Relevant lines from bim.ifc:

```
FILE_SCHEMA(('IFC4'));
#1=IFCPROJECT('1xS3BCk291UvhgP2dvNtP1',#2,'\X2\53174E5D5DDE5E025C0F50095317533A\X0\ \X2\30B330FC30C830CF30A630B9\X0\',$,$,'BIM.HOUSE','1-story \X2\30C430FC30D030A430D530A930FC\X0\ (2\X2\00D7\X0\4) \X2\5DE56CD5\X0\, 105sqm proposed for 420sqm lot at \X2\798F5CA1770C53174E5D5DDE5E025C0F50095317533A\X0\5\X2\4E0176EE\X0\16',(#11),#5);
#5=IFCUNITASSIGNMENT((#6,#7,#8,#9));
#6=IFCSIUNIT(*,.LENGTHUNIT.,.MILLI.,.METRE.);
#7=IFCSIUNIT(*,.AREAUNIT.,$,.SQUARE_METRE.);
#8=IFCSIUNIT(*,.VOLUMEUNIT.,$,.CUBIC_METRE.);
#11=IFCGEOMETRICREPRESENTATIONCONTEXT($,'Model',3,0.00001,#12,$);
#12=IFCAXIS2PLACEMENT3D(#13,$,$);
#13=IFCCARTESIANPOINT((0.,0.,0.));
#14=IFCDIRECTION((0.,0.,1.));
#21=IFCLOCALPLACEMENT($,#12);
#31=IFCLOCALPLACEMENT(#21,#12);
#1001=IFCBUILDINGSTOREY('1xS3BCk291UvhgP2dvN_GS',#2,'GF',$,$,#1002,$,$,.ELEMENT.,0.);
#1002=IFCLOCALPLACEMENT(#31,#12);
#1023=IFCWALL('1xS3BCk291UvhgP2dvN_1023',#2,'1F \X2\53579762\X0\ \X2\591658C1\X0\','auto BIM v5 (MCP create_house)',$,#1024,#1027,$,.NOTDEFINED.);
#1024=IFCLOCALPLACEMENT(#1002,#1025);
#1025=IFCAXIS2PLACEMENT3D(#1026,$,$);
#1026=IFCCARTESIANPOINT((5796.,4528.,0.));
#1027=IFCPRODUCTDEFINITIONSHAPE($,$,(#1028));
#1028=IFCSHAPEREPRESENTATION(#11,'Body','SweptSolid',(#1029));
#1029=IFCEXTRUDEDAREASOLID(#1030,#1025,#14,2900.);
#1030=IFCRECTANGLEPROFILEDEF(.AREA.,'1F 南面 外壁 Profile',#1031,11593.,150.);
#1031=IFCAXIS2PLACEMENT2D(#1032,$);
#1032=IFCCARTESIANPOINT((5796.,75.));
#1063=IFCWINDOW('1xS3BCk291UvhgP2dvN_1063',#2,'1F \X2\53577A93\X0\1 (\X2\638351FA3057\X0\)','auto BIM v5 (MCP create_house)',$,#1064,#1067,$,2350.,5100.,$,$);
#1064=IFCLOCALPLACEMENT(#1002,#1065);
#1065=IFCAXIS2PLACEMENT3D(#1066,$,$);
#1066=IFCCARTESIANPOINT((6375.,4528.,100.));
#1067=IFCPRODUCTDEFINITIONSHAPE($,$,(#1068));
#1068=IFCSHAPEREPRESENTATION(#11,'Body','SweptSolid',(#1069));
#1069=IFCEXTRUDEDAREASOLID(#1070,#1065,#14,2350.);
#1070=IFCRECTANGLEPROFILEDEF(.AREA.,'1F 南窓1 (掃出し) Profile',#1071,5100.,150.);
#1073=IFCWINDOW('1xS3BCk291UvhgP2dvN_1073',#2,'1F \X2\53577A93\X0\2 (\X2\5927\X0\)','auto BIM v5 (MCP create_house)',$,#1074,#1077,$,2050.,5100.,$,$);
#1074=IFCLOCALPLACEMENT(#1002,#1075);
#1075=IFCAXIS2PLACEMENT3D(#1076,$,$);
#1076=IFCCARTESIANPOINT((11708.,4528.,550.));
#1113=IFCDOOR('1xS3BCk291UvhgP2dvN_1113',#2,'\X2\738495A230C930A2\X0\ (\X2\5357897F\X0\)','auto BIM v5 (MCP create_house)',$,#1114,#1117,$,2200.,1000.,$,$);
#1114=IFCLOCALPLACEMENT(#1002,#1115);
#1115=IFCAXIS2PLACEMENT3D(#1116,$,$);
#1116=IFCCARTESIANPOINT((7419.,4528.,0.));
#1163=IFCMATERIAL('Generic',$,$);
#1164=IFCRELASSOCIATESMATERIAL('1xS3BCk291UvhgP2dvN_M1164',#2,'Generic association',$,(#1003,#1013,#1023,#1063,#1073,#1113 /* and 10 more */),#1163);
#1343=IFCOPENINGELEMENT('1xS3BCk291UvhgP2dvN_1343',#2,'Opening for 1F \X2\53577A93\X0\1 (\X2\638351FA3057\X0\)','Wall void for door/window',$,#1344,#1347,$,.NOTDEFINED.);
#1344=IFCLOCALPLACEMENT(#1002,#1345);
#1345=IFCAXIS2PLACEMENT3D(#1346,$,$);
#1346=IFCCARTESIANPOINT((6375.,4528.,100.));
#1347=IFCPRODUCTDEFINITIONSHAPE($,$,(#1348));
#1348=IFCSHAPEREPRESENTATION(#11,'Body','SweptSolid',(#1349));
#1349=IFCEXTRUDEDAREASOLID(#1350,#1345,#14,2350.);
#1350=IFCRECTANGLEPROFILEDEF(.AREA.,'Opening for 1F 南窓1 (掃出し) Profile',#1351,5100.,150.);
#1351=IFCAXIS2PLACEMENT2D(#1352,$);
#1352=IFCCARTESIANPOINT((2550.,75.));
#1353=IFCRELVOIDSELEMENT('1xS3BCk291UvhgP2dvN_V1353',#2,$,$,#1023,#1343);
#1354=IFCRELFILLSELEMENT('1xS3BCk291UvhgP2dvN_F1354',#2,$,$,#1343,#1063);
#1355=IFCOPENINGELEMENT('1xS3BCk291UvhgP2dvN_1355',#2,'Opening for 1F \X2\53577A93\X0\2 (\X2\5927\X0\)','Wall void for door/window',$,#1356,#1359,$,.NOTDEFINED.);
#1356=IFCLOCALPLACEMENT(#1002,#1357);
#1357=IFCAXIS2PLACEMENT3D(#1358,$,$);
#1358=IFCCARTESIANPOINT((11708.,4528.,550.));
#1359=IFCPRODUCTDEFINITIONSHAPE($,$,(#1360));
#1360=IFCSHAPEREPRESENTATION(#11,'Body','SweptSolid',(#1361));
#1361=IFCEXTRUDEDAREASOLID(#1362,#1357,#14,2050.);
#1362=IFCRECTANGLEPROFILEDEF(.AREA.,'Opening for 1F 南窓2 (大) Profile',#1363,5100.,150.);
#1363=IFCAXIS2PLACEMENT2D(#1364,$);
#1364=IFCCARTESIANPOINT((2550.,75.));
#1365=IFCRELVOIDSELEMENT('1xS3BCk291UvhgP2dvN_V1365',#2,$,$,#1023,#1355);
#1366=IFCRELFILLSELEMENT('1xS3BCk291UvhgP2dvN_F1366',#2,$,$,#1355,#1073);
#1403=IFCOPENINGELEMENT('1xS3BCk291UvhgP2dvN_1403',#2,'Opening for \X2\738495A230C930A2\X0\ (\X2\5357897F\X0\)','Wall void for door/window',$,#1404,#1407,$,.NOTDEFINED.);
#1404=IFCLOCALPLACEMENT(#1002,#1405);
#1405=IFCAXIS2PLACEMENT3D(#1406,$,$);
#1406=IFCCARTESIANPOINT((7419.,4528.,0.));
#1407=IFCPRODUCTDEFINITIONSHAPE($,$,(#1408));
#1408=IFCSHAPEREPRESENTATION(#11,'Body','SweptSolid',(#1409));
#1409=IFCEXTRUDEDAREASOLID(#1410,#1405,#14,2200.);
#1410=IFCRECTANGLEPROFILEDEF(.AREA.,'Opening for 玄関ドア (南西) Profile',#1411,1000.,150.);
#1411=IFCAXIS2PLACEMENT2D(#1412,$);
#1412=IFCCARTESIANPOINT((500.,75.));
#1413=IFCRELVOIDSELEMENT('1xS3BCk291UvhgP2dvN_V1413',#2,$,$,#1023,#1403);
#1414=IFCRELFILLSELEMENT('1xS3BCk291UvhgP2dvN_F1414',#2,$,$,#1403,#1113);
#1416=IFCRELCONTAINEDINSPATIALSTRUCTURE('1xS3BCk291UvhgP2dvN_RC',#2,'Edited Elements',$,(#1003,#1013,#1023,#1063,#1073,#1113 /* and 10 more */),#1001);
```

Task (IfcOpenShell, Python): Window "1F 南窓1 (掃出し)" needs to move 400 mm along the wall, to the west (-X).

```python
import ifcopenshell
import ifcopenshell.api.geometry
import ifcopenshell.util.placement
import ifcopenshell.util.unit

model = ifcopenshell.open("bim.ifc")
unit_scale = ifcopenshell.util.unit.calculate_unit_scale(model)

window = model.by_guid("1xS3BCk291UvhgP2dvN_1063")
opening = window.FillsVoids[0].RelatingOpeningElement
wall = opening.VoidsElements[0].RelatingBuildingElement

wall_matrix = ifcopenshell.util.placement.get_local_placement(wall.ObjectPlacement)
shift = wall_matrix[:3, 0] * -0.4 / unit_scale
before = ifcopenshell.util.placement.get_local_placement(window.ObjectPlacement)[:3, 3].copy()

# The window is not placed relative to its opening, so move both.
for product in (opening, window):
    matrix = ifcopenshell.util.placement.get_local_placement(product.ObjectPlacement)
    matrix[:3, 3] += shift
    ifcopenshell.api.geometry.edit_object_placement(model, product=product, matrix=matrix, is_si=False)

after = ifcopenshell.util.placement.get_local_placement(window.ObjectPlacement)[:3, 3]
print("window moved by", (after - before).round(3) + 0.0)

model.write("bim_v2.ifc")
```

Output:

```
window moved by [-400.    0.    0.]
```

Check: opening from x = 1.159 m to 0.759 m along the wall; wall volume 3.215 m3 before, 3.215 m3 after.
